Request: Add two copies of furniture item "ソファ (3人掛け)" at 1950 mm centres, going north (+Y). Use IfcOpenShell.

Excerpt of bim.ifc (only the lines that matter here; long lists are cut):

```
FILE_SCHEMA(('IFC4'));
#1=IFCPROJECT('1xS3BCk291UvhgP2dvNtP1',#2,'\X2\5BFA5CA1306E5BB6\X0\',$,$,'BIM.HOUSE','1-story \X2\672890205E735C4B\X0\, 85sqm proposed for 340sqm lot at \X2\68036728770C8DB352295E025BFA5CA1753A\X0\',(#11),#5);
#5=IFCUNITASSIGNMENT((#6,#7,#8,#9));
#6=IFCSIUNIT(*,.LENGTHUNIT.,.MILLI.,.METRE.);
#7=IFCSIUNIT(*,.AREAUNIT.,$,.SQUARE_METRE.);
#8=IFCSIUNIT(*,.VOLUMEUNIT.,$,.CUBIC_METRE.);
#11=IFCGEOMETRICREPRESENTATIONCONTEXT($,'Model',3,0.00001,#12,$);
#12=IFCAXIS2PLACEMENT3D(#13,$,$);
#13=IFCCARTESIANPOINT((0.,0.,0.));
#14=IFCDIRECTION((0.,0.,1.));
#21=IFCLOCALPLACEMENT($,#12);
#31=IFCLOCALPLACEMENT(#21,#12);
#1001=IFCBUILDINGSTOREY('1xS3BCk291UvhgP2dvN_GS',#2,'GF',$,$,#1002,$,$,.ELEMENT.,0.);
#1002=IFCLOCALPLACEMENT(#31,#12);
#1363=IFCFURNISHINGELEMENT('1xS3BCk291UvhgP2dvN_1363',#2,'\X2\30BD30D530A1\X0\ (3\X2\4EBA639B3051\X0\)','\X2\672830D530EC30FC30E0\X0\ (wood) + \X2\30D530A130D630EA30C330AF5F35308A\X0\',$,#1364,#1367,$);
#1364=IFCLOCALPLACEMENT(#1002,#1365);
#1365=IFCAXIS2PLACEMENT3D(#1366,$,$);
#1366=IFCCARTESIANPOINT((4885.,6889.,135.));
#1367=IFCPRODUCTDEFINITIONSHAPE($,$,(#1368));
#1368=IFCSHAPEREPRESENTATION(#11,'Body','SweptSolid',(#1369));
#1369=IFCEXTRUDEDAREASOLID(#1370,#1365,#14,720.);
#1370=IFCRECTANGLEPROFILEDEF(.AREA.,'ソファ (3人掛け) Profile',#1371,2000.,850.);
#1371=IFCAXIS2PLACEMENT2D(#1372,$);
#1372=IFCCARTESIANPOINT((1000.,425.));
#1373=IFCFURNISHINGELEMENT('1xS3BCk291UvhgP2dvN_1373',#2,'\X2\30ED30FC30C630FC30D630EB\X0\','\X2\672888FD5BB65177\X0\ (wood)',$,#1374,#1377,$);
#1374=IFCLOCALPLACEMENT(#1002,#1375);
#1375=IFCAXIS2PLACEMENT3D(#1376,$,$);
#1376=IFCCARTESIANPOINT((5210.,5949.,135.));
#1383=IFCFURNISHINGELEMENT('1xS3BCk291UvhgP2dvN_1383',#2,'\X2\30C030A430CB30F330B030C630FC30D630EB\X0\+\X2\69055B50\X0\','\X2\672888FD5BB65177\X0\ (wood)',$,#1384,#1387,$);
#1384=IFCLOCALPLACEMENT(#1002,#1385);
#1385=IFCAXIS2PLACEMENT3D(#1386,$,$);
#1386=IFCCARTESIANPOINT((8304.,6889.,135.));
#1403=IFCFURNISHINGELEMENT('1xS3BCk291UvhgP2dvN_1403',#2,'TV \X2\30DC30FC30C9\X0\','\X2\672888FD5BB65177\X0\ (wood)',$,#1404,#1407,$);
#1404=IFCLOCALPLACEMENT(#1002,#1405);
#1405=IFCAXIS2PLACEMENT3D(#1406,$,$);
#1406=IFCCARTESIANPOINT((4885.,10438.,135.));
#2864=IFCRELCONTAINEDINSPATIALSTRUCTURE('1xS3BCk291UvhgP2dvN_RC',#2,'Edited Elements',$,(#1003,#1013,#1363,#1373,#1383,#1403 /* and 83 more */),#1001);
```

```python
import numpy as np
import ifcopenshell
import ifcopenshell.api.geometry
import ifcopenshell.api.root
import ifcopenshell.util.element
import ifcopenshell.util.placement
import ifcopenshell.util.unit

model = ifcopenshell.open("bim.ifc")
unit_scale = ifcopenshell.util.unit.calculate_unit_scale(model)


def reuse_history(source, copy):
    """copy_class also copies each property set's owner history, people and application; keep the originals."""
    for rel in copy.IsDefinedBy:
        if rel.is_a("IfcRelDefinesByProperties") and (history := rel.RelatingPropertyDefinition.OwnerHistory):
            rel.RelatingPropertyDefinition.OwnerHistory = source.OwnerHistory
            ifcopenshell.util.element.remove_deep2(model, history)


source = model.by_guid("1xS3BCk291UvhgP2dvN_1363")
base = ifcopenshell.util.placement.get_local_placement(source.ObjectPlacement)
step = np.array([0.0, 1.0, 0.0]) * 1.95 / unit_scale

for i in range(1, 3):
    copy = ifcopenshell.api.root.copy_class(model, product=source)
    copy.Representation = ifcopenshell.util.element.copy_deep(
        model, source.Representation, exclude=["IfcGeometricRepresentationContext", "IfcRepresentationMap"]
    )
    reuse_history(source, copy)
    matrix = base.copy()
    matrix[:3, 3] += i * step
    print("added at", matrix[:3, 3].round(3) + 0.0)
    ifcopenshell.api.geometry.edit_object_placement(model, product=copy, matrix=matrix, is_si=False)

model.write("bim-out.ifc")
```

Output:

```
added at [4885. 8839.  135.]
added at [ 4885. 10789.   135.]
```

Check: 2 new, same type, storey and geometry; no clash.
